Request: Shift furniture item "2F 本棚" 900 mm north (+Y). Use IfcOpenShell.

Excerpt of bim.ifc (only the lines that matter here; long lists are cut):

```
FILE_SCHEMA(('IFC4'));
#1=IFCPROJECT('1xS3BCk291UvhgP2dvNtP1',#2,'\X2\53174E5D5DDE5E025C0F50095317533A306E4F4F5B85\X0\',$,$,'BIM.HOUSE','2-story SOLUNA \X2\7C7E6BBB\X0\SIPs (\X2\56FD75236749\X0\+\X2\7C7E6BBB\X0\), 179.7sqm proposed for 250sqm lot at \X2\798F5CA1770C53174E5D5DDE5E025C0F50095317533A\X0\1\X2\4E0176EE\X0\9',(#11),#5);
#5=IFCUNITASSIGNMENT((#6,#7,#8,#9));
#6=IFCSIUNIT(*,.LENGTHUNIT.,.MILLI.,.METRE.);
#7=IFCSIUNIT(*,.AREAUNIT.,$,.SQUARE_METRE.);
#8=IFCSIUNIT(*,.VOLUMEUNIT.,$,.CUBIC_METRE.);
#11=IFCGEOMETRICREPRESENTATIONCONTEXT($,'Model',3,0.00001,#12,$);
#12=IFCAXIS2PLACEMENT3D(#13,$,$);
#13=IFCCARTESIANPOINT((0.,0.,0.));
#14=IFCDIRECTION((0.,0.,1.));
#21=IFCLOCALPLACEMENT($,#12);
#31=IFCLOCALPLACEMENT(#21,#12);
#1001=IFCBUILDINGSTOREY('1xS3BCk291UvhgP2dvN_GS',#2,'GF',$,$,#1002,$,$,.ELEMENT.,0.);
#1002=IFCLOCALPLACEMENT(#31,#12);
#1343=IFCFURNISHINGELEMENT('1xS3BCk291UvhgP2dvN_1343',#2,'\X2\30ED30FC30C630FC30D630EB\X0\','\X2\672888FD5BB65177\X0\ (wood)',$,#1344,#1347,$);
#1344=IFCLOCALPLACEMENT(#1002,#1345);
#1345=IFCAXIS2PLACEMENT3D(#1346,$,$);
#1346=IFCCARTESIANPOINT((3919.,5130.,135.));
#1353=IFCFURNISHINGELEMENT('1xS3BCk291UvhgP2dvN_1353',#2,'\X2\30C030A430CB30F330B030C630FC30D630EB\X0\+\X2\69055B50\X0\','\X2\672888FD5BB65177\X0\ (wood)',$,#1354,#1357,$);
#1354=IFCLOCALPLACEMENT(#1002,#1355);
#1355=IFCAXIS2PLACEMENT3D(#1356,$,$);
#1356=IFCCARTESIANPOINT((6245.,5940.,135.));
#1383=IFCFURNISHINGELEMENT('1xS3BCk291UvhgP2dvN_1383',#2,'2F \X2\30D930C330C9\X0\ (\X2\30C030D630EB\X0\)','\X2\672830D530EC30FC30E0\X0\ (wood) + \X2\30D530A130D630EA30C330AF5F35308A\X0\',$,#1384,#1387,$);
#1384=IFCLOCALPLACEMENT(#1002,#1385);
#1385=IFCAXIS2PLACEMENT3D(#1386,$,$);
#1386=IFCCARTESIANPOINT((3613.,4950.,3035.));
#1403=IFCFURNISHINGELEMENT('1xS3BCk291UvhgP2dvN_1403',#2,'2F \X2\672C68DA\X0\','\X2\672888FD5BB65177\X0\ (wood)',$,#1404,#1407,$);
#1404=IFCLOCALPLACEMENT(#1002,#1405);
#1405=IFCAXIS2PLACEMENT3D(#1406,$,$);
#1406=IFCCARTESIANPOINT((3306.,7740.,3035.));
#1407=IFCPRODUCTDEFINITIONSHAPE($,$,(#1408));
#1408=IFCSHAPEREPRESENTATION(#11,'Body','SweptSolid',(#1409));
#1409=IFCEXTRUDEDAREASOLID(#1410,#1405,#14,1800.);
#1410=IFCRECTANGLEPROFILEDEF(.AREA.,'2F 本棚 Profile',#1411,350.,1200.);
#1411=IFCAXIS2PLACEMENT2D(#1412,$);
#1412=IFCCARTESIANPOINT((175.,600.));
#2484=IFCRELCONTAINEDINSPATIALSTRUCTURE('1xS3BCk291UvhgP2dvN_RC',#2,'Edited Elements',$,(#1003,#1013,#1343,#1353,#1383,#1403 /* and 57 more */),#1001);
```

```python
import ifcopenshell
import ifcopenshell.api.geometry
import ifcopenshell.util.placement

model = ifcopenshell.open("bim.ifc")

item = model.by_guid("1xS3BCk291UvhgP2dvN_1403")
matrix = ifcopenshell.util.placement.get_local_placement(item.ObjectPlacement)
matrix[1, 3] += 900.0
ifcopenshell.api.geometry.edit_object_placement(model, product=item, matrix=matrix, is_si=False)

print(ifcopenshell.util.placement.get_local_placement(item.ObjectPlacement).round(3) + 0.0)

model.write("bim_v2.ifc")
```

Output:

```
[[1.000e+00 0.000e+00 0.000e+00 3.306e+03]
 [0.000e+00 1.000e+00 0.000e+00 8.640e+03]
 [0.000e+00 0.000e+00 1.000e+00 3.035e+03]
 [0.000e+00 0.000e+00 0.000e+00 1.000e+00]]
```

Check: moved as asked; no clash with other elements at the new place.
